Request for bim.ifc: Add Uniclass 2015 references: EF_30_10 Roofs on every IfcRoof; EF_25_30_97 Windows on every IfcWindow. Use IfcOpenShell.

First a look at what the model holds.

```python
import ifcopenshell

model = ifcopenshell.open("bim.ifc")
print(model.schema)
print("classifications:", [c.Name for c in model.by_type("IfcClassification")])
for ifc_class in ("IfcDoor", "IfcRoof", "IfcStair", "IfcWall", "IfcWindow"):
    print(ifc_class, len(model.by_type(ifc_class)))
```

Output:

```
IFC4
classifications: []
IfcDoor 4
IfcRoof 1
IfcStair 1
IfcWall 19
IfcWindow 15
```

```python
import ifcopenshell
import ifcopenshell.api.classification

model = ifcopenshell.open("bim.ifc")

system = ifcopenshell.api.classification.add_classification(model, classification="Uniclass 2015")

codes = {
    "IfcRoof": ("EF_30_10", "Roofs"),
    "IfcWindow": ("EF_25_30_97", "Windows"),
}
for ifc_class, (code, name) in codes.items():
    products = model.by_type(ifc_class)
    ifcopenshell.api.classification.add_reference(
        model, products=products, classification=system, identification=code, name=name
    )
    print(code, len(products))

model.write("bim_rev.ifc")
```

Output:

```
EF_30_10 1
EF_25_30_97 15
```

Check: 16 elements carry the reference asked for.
